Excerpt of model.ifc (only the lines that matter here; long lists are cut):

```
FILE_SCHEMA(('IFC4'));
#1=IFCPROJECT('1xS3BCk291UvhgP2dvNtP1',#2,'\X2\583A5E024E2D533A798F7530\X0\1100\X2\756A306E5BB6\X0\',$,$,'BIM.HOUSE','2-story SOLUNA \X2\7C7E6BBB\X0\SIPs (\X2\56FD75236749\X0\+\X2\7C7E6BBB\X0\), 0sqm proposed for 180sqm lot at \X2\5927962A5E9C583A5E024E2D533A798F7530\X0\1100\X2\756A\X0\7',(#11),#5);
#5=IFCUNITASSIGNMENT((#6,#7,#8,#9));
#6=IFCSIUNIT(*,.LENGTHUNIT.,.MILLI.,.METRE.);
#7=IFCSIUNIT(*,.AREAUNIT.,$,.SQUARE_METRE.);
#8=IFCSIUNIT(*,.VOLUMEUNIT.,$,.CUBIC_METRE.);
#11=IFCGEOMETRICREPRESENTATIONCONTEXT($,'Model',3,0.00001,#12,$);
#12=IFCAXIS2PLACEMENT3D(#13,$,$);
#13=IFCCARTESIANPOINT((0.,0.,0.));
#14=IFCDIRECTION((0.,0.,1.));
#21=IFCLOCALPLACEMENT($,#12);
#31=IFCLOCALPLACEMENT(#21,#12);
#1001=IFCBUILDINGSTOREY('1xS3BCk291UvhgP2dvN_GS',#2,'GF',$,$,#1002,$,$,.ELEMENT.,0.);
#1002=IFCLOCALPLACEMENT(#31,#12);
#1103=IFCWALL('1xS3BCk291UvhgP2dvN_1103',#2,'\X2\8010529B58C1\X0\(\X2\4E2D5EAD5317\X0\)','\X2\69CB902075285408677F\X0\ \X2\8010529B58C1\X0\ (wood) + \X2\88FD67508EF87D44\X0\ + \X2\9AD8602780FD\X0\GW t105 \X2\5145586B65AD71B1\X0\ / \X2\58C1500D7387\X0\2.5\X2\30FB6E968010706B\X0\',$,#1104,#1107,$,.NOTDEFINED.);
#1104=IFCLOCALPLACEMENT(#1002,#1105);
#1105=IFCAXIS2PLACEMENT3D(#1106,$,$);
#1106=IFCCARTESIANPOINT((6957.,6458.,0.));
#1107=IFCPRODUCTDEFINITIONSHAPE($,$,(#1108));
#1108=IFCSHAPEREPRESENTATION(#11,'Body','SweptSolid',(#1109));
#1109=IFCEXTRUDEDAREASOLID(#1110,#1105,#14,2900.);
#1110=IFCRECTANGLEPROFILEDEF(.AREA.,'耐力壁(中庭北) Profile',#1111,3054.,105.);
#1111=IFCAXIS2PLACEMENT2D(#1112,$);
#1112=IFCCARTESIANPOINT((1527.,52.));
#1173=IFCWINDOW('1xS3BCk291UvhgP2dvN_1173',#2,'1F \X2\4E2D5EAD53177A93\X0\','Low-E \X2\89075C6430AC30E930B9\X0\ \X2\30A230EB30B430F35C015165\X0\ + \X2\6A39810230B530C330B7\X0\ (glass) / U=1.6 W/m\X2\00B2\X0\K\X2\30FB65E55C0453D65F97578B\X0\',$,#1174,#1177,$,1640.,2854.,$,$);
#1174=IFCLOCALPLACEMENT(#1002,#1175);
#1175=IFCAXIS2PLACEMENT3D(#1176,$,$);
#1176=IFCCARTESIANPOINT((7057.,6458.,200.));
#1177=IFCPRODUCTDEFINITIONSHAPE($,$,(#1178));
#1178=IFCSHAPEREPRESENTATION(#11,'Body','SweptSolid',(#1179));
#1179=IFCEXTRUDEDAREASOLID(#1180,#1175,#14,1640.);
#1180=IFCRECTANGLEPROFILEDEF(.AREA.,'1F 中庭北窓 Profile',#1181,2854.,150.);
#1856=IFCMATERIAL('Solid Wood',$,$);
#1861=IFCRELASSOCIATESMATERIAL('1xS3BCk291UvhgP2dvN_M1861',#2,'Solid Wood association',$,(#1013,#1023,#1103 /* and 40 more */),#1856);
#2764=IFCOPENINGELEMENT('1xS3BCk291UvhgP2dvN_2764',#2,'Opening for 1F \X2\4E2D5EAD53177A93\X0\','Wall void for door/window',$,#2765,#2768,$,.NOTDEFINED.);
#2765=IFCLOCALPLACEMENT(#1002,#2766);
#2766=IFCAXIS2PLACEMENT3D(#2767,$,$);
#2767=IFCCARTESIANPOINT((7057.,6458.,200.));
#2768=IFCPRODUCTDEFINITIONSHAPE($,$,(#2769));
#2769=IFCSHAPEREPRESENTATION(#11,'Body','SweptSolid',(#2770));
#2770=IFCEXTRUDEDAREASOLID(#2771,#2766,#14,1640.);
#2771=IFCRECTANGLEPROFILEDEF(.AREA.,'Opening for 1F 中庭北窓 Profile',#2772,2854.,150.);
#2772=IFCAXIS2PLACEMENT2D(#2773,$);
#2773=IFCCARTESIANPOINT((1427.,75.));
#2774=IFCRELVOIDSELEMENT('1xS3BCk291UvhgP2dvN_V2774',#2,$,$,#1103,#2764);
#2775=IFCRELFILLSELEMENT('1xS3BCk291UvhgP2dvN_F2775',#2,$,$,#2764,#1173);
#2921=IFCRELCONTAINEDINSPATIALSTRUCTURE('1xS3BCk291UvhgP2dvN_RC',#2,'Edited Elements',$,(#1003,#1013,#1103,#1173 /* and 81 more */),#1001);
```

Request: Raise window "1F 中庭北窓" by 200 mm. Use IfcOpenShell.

```python
import numpy as np
import ifcopenshell
import ifcopenshell.api.geometry
import ifcopenshell.util.placement
import ifcopenshell.util.unit

model = ifcopenshell.open("model.ifc")
unit_scale = ifcopenshell.util.unit.calculate_unit_scale(model)

window = model.by_guid("1xS3BCk291UvhgP2dvN_1173")
opening = window.FillsVoids[0].RelatingOpeningElement
dz = 200.0

shift = np.array([0.0, 0.0, dz])
# The window is not placed relative to its opening, so move both.
for product in (opening, window):
    matrix = ifcopenshell.util.placement.get_local_placement(product.ObjectPlacement)
    matrix[:3, 3] += shift
    ifcopenshell.api.geometry.edit_object_placement(model, product=product, matrix=matrix, is_si=False)

print(f"moved by {dz * unit_scale:+.3f} m")

model.write("model-out.ifc")
```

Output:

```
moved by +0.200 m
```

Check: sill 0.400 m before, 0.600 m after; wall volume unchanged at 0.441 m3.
